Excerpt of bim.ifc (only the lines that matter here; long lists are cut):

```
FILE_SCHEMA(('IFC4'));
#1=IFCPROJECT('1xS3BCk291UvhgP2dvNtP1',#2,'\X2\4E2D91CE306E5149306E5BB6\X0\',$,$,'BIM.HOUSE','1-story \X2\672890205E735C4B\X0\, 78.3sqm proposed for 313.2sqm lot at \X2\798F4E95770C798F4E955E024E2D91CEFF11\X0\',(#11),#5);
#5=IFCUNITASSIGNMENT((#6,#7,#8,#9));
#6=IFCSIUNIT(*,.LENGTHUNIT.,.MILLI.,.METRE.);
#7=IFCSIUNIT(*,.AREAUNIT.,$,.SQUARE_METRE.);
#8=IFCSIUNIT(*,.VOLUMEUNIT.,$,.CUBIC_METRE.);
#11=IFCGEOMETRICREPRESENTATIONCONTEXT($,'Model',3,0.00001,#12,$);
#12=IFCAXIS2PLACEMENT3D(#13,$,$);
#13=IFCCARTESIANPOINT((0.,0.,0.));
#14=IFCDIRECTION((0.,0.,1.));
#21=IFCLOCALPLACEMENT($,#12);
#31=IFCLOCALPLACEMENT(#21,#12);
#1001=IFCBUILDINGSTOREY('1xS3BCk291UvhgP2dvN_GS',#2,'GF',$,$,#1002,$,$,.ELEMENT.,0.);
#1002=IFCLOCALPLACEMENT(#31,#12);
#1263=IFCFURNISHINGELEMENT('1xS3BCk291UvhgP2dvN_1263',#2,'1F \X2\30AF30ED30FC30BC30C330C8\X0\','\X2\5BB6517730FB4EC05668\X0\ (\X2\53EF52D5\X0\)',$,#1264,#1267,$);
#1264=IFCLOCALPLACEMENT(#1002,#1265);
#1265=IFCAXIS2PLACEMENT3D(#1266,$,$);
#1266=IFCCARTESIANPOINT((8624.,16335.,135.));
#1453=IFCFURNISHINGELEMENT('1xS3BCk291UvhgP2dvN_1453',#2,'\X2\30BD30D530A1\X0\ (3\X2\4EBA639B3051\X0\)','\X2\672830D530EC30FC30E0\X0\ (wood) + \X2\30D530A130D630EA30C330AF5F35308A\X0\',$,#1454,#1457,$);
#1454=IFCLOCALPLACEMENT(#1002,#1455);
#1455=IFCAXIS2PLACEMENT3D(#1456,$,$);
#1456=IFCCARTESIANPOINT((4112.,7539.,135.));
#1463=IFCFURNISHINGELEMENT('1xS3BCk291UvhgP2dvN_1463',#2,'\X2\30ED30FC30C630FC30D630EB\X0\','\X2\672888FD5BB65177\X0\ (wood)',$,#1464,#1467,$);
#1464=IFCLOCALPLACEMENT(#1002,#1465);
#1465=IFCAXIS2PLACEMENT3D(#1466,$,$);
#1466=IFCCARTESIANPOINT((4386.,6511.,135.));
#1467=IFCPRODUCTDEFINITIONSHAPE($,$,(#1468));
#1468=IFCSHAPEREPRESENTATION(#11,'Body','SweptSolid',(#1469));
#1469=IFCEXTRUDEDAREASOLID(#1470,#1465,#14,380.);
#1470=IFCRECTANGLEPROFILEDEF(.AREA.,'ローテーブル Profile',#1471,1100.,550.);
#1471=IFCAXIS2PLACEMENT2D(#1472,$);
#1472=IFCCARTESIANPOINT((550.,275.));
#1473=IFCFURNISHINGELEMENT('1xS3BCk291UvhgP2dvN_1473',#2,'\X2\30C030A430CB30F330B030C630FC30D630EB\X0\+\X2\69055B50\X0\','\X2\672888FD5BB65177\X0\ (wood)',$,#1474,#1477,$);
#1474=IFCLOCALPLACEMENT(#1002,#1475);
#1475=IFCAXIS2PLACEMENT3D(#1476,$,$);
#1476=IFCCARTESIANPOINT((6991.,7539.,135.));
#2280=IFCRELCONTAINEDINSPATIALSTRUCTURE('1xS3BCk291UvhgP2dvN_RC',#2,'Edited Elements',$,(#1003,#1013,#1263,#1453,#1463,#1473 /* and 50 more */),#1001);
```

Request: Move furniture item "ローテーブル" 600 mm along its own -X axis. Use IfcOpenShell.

```python
import ifcopenshell
import ifcopenshell.api.geometry
import ifcopenshell.util.placement

model = ifcopenshell.open("bim.ifc")

item = model.by_id(1463)
matrix = ifcopenshell.util.placement.get_local_placement(item.ObjectPlacement)
matrix[:3, 3] -= matrix[:3, 0] * 600.0
ifcopenshell.api.geometry.edit_object_placement(model, product=item, matrix=matrix, is_si=False)

print(ifcopenshell.util.placement.get_local_placement(item.ObjectPlacement).round(3) + 0.0)

model.write("bim_edited.ifc")
```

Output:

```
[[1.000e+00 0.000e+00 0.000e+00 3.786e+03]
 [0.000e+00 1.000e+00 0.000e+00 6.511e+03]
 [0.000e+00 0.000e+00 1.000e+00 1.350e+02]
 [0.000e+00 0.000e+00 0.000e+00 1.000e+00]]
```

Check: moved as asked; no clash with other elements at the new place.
